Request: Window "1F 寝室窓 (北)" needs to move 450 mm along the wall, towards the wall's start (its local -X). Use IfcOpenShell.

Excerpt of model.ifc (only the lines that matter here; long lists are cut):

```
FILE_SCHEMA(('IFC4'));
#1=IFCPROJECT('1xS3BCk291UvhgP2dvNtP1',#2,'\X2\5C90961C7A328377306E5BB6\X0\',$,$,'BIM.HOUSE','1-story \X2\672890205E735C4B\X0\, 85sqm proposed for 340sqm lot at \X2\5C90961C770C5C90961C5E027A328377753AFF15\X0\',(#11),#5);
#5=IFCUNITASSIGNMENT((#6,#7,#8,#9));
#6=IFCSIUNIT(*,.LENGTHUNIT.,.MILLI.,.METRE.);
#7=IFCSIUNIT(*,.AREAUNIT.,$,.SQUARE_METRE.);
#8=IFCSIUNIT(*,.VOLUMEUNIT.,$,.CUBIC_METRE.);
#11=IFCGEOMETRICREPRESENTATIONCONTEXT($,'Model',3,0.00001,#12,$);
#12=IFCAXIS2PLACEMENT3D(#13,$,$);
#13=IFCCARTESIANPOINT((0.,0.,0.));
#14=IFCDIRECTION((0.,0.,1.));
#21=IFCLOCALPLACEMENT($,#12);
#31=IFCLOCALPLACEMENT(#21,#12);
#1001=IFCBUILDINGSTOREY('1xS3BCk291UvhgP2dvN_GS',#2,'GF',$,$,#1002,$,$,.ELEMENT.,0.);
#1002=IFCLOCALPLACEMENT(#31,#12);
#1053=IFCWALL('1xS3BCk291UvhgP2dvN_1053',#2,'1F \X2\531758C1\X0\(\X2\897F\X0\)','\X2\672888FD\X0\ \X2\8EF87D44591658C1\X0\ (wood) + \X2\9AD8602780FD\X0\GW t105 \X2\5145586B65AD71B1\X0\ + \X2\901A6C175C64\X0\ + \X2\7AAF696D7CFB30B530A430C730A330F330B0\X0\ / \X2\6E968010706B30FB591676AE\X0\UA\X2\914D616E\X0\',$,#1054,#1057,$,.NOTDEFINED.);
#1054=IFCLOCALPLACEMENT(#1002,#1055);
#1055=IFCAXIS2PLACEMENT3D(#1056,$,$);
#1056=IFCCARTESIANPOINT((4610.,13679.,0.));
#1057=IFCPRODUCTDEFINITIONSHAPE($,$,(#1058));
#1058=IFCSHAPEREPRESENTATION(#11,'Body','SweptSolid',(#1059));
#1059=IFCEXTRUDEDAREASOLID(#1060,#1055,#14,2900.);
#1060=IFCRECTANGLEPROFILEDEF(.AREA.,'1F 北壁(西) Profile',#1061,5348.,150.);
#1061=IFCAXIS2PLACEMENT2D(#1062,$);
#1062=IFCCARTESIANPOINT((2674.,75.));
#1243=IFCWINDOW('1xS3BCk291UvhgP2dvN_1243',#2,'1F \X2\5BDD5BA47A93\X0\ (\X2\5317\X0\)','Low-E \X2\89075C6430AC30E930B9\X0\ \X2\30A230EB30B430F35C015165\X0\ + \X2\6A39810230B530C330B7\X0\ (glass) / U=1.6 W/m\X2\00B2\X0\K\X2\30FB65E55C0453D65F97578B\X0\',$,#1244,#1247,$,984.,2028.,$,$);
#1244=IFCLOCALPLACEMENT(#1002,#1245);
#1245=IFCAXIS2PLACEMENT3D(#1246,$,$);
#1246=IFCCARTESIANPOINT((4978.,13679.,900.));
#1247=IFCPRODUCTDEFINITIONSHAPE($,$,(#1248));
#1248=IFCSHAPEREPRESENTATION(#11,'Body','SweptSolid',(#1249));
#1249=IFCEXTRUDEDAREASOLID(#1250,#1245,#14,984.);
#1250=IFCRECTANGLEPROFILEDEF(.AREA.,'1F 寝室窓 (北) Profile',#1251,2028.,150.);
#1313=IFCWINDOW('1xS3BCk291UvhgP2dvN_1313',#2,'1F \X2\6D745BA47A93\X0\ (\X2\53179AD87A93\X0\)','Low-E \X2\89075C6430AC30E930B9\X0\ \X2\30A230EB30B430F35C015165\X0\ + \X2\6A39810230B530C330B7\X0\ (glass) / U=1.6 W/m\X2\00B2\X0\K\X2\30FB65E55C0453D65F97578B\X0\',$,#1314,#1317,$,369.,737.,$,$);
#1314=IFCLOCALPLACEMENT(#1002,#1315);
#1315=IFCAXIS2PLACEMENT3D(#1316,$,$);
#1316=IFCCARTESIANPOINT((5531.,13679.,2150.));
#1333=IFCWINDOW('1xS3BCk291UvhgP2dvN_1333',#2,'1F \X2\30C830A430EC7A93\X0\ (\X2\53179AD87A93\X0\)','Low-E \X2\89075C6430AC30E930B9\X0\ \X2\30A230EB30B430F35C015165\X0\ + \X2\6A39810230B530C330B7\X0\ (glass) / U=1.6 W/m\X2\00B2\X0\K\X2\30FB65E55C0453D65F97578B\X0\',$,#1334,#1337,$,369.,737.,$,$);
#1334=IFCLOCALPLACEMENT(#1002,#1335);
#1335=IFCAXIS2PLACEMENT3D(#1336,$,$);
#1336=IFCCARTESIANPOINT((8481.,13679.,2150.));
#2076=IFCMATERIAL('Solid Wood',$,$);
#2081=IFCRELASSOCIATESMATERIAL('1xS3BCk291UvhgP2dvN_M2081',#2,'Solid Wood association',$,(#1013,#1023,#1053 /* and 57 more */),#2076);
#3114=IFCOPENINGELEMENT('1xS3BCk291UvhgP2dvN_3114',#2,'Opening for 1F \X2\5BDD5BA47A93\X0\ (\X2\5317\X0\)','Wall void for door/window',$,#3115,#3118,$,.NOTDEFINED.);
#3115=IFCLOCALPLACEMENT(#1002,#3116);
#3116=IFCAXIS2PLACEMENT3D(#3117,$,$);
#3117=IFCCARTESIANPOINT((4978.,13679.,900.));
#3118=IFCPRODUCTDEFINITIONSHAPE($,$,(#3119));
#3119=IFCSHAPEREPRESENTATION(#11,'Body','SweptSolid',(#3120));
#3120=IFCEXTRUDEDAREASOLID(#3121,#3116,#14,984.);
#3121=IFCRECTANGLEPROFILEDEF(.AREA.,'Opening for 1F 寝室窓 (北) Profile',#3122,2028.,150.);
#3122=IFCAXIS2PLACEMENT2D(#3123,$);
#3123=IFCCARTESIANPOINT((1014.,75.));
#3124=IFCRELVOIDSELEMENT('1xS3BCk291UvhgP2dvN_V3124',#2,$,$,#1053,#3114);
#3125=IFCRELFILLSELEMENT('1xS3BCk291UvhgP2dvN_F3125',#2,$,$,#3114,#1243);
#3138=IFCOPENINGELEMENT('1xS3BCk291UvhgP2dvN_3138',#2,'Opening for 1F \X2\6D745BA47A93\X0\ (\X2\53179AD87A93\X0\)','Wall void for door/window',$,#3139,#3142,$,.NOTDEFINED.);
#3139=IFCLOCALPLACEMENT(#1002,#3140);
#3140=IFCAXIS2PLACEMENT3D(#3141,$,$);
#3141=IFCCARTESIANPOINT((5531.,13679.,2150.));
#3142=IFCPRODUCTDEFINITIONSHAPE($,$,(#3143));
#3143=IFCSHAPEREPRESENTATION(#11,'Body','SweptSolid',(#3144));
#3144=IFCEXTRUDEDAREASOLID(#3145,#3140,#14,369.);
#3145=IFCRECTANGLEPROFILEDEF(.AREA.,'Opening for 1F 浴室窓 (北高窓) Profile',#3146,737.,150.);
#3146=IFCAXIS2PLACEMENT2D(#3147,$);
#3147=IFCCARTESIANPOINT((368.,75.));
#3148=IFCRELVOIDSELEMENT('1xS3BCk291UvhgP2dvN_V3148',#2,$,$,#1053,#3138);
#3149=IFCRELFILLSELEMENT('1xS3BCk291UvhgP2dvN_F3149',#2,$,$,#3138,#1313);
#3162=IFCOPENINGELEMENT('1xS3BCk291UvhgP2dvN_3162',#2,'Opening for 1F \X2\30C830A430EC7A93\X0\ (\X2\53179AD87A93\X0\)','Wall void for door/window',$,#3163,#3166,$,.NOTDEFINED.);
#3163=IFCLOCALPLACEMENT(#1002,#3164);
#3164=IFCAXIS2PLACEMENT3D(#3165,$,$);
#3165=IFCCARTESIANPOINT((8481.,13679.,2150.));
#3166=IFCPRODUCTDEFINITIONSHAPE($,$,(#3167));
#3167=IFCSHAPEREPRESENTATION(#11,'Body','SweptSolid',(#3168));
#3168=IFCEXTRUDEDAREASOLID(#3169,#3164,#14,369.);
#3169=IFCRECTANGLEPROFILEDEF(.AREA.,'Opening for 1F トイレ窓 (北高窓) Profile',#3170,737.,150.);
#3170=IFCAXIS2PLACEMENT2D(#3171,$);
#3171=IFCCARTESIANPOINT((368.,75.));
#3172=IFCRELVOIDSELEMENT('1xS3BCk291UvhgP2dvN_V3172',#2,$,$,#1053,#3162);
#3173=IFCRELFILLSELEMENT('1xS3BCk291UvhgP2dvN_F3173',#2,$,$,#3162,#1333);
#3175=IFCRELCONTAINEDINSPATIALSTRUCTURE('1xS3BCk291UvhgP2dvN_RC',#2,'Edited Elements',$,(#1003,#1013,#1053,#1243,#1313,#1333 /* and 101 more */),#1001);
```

```python
import ifcopenshell
import ifcopenshell.api.geometry
import ifcopenshell.util.placement

model = ifcopenshell.open("model.ifc")

window = model.by_guid("1xS3BCk291UvhgP2dvN_1243")
opening = window.FillsVoids[0].RelatingOpeningElement
wall = opening.VoidsElements[0].RelatingBuildingElement

wall_matrix = ifcopenshell.util.placement.get_local_placement(wall.ObjectPlacement)
shift = wall_matrix[:3, 0] * -450.0
before = ifcopenshell.util.placement.get_local_placement(window.ObjectPlacement)[:3, 3].copy()

# The window is not placed relative to its opening, so move both.
for product in (opening, window):
    matrix = ifcopenshell.util.placement.get_local_placement(product.ObjectPlacement)
    matrix[:3, 3] += shift
    ifcopenshell.api.geometry.edit_object_placement(model, product=product, matrix=matrix, is_si=False)

after = ifcopenshell.util.placement.get_local_placement(window.ObjectPlacement)[:3, 3]
print("window moved by", (after - before).round(3) + 0.0)

model.write("model_v2.ifc")
```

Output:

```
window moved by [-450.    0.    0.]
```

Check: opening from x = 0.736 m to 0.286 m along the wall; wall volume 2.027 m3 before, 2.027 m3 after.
